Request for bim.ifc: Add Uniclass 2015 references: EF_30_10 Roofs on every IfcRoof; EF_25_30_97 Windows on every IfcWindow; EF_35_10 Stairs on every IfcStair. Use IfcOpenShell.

First a look at what the model holds.

```python
import ifcopenshell

model = ifcopenshell.open("bim.ifc")
print(model.schema)
print("classifications:", [c.Name for c in model.by_type("IfcClassification")])
for ifc_class in ("IfcDoor", "IfcRoof", "IfcStair", "IfcWall", "IfcWindow"):
    print(ifc_class, len(model.by_type(ifc_class)))
```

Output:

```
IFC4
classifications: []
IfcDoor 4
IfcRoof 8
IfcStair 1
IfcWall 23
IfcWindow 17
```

```python
import ifcopenshell
import ifcopenshell.api.classification

model = ifcopenshell.open("bim.ifc")

system = ifcopenshell.api.classification.add_classification(model, classification="Uniclass 2015")

codes = {
    "IfcRoof": ("EF_30_10", "Roofs"),
    "IfcWindow": ("EF_25_30_97", "Windows"),
    "IfcStair": ("EF_35_10", "Stairs"),
}
for ifc_class, (code, name) in codes.items():
    products = model.by_type(ifc_class)
    ifcopenshell.api.classification.add_reference(
        model, products=products, classification=system, identification=code, name=name
    )
    print(code, len(products))

model.write("bim_rev.ifc")
```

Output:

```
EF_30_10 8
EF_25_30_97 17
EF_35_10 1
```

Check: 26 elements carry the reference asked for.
